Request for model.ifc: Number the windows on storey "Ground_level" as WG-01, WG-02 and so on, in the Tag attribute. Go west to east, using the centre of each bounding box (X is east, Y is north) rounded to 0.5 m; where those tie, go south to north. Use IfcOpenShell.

First a look at what the model holds.

```python
import ifcopenshell
import ifcopenshell.util.element
import ifcopenshell.util.placement

model = ifcopenshell.open("model.ifc")
print(model.schema)
storey = next(s for s in model.by_type("IfcBuildingStorey") if s.Name == "Ground_level")
windows = [e for e in ifcopenshell.util.element.get_decomposition(storey) if e.is_a("IfcWindow")]
for e in sorted(windows, key=lambda e: e.id()):
    origin = ifcopenshell.util.placement.get_local_placement(e.ObjectPlacement)[:3, 3]
    print(e.id(), e.Tag, e.Name, origin.round(2) + 0.0, sep=" | ")
```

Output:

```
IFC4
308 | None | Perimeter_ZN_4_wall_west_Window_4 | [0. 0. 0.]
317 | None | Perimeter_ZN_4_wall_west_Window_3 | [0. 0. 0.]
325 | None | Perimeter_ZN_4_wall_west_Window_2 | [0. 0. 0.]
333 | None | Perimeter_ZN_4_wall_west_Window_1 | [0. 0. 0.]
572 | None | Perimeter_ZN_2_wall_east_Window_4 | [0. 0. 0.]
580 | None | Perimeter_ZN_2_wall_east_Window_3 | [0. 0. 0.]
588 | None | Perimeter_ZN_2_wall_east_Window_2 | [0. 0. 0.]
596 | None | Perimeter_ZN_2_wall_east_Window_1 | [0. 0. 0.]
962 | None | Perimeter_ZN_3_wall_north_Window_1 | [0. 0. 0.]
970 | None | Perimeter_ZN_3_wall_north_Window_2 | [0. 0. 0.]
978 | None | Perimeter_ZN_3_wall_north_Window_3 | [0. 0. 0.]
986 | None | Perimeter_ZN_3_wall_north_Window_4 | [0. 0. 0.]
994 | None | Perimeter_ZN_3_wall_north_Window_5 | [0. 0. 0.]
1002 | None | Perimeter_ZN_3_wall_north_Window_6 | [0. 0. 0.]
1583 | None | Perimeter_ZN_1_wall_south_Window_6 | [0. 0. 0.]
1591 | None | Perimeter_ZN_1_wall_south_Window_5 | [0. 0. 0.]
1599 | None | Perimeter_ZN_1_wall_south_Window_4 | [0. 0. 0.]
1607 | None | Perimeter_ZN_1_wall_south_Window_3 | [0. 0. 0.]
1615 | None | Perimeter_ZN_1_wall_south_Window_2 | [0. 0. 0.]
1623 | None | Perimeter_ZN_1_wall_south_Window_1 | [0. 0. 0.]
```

```python
import ifcopenshell
import ifcopenshell.geom
import ifcopenshell.util.element
import ifcopenshell.util.shape

model = ifcopenshell.open("model.ifc")
settings = ifcopenshell.geom.settings()
settings.set("use-world-coords", True)


def centre(element):
    shape = ifcopenshell.geom.create_shape(settings, element)
    return ifcopenshell.util.shape.get_bbox_centroid(shape.geometry)


storey = next(s for s in model.by_type("IfcBuildingStorey") if s.Name == "Ground_level")
windows = [e for e in ifcopenshell.util.element.get_decomposition(storey) if e.is_a("IfcWindow")]

# Insertion points can sit at a corner or the storey origin, so sort by the geometry (in metres).
centres = {e: centre(e) for e in windows}
windows.sort(key=lambda e: (round(centres[e][0] / 0.5), centres[e][1]))

for i, e in enumerate(windows, start=1):
    number = f"WG-{i:02d}"
    e.Tag = number
    print(e.id(), number)

model.write("model_rev.ifc")
```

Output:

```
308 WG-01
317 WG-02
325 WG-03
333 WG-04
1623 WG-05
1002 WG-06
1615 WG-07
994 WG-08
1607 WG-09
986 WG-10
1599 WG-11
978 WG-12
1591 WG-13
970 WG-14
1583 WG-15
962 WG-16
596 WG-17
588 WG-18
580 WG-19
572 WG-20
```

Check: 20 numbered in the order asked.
